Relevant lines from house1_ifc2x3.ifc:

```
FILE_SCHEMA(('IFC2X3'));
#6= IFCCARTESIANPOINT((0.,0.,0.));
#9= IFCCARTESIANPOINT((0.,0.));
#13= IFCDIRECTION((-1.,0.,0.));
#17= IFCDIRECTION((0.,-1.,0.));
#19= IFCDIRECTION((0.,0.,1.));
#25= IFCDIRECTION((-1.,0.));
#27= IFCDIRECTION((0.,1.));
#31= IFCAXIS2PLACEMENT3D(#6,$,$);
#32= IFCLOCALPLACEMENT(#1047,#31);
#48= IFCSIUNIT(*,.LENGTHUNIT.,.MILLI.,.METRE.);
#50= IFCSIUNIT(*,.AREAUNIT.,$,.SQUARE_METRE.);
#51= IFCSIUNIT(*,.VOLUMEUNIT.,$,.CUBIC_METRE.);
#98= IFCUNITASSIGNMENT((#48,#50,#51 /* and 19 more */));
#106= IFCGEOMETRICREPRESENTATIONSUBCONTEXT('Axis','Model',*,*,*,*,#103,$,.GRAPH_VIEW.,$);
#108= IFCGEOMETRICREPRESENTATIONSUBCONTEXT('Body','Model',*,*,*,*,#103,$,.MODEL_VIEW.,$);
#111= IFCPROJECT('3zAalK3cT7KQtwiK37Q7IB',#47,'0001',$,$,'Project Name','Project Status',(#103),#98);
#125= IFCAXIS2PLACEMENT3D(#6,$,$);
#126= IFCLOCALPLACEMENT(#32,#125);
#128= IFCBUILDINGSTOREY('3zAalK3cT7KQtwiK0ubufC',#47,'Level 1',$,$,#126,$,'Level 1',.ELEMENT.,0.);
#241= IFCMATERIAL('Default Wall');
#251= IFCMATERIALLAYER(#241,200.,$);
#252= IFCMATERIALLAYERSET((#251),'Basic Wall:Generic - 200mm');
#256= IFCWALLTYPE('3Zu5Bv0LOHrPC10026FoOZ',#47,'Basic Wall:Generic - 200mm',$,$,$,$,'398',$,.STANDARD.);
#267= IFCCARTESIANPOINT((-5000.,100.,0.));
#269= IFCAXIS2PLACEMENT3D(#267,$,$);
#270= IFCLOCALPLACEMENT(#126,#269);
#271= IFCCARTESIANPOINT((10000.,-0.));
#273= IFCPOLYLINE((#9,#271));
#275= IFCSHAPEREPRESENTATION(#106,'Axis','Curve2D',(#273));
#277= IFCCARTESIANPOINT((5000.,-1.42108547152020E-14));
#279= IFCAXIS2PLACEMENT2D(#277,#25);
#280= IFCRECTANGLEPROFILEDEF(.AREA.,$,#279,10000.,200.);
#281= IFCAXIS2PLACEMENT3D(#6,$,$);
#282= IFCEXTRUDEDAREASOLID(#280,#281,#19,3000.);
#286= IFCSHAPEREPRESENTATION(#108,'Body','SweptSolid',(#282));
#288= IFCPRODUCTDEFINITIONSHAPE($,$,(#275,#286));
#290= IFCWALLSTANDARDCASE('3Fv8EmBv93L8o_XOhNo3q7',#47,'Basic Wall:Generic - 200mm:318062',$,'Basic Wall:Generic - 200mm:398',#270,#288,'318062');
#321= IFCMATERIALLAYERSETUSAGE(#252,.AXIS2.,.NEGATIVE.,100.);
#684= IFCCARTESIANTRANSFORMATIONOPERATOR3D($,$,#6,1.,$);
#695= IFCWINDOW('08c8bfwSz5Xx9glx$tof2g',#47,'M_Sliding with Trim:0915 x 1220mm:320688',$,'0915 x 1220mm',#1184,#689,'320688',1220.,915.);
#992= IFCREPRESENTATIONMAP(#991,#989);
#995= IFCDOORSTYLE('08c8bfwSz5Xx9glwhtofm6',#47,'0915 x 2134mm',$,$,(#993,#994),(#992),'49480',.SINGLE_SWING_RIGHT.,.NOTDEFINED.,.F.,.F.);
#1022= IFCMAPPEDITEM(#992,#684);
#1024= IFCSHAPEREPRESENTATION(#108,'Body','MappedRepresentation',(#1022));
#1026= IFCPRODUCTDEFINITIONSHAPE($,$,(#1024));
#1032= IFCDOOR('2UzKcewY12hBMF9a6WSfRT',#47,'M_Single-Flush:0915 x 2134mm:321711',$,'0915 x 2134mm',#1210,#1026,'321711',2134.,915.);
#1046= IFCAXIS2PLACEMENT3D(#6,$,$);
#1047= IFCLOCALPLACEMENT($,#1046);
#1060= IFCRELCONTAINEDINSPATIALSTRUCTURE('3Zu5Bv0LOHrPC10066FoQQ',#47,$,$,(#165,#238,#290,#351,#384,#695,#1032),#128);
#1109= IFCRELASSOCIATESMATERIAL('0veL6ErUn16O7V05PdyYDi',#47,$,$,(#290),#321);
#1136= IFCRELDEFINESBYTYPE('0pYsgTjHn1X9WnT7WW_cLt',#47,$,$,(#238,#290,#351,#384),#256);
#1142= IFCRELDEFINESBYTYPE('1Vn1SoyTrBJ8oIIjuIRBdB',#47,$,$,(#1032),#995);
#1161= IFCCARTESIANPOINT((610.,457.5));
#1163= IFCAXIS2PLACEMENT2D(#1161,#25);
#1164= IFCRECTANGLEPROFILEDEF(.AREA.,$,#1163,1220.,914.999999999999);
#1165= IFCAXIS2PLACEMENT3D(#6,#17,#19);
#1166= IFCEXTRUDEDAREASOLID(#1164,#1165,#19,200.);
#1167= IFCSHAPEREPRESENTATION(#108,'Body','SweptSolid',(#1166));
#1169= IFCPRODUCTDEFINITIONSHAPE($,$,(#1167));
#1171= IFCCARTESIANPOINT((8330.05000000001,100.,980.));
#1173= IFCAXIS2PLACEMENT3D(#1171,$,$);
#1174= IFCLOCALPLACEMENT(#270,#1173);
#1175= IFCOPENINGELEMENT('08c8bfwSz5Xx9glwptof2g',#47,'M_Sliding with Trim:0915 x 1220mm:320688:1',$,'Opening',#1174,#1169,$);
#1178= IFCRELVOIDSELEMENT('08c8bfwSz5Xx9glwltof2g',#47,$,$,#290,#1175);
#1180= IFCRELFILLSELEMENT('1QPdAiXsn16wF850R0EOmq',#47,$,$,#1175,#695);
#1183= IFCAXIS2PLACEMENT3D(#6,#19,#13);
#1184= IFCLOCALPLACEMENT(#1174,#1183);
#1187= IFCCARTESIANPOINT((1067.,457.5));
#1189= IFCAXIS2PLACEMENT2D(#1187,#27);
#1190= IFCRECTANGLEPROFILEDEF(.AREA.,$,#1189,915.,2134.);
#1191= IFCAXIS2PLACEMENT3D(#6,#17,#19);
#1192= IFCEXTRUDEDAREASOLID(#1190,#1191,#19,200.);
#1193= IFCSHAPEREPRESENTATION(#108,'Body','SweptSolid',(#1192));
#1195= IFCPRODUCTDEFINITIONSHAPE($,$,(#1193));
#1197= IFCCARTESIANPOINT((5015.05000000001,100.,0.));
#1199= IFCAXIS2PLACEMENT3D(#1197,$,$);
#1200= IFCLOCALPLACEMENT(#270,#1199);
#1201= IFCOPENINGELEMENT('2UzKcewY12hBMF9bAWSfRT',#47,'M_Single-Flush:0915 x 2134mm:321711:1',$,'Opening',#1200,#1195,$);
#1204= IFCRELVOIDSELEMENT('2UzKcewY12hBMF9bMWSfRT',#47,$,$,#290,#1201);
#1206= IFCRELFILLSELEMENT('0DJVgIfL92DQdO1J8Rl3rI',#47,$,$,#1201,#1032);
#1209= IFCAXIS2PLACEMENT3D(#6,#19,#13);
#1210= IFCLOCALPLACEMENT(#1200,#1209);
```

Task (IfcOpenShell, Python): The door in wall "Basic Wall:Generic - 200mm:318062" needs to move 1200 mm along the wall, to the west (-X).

```python
import ifcopenshell
import ifcopenshell.api.geometry
import ifcopenshell.util.placement
import ifcopenshell.util.unit

model = ifcopenshell.open("house1_ifc2x3.ifc")
unit_scale = ifcopenshell.util.unit.calculate_unit_scale(model)

door = model.by_id(1032)
opening = door.FillsVoids[0].RelatingOpeningElement
wall = opening.VoidsElements[0].RelatingBuildingElement

wall_matrix = ifcopenshell.util.placement.get_local_placement(wall.ObjectPlacement)
shift = wall_matrix[:3, 0] * -1.2 / unit_scale
before = ifcopenshell.util.placement.get_local_placement(door.ObjectPlacement)[:3, 3].copy()

# The door is placed relative to its opening, so it follows when the opening moves.
matrix = ifcopenshell.util.placement.get_local_placement(opening.ObjectPlacement)
matrix[:3, 3] += shift
ifcopenshell.api.geometry.edit_object_placement(
    model, product=opening, matrix=matrix, is_si=False, should_transform_children=True
)

after = ifcopenshell.util.placement.get_local_placement(door.ObjectPlacement)[:3, 3]
print("door moved by", (after - before).round(3) + 0.0)

model.write("house1_ifc2x3_updated.ifc")
```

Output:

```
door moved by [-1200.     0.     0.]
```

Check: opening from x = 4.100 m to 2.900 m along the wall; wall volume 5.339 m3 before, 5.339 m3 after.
